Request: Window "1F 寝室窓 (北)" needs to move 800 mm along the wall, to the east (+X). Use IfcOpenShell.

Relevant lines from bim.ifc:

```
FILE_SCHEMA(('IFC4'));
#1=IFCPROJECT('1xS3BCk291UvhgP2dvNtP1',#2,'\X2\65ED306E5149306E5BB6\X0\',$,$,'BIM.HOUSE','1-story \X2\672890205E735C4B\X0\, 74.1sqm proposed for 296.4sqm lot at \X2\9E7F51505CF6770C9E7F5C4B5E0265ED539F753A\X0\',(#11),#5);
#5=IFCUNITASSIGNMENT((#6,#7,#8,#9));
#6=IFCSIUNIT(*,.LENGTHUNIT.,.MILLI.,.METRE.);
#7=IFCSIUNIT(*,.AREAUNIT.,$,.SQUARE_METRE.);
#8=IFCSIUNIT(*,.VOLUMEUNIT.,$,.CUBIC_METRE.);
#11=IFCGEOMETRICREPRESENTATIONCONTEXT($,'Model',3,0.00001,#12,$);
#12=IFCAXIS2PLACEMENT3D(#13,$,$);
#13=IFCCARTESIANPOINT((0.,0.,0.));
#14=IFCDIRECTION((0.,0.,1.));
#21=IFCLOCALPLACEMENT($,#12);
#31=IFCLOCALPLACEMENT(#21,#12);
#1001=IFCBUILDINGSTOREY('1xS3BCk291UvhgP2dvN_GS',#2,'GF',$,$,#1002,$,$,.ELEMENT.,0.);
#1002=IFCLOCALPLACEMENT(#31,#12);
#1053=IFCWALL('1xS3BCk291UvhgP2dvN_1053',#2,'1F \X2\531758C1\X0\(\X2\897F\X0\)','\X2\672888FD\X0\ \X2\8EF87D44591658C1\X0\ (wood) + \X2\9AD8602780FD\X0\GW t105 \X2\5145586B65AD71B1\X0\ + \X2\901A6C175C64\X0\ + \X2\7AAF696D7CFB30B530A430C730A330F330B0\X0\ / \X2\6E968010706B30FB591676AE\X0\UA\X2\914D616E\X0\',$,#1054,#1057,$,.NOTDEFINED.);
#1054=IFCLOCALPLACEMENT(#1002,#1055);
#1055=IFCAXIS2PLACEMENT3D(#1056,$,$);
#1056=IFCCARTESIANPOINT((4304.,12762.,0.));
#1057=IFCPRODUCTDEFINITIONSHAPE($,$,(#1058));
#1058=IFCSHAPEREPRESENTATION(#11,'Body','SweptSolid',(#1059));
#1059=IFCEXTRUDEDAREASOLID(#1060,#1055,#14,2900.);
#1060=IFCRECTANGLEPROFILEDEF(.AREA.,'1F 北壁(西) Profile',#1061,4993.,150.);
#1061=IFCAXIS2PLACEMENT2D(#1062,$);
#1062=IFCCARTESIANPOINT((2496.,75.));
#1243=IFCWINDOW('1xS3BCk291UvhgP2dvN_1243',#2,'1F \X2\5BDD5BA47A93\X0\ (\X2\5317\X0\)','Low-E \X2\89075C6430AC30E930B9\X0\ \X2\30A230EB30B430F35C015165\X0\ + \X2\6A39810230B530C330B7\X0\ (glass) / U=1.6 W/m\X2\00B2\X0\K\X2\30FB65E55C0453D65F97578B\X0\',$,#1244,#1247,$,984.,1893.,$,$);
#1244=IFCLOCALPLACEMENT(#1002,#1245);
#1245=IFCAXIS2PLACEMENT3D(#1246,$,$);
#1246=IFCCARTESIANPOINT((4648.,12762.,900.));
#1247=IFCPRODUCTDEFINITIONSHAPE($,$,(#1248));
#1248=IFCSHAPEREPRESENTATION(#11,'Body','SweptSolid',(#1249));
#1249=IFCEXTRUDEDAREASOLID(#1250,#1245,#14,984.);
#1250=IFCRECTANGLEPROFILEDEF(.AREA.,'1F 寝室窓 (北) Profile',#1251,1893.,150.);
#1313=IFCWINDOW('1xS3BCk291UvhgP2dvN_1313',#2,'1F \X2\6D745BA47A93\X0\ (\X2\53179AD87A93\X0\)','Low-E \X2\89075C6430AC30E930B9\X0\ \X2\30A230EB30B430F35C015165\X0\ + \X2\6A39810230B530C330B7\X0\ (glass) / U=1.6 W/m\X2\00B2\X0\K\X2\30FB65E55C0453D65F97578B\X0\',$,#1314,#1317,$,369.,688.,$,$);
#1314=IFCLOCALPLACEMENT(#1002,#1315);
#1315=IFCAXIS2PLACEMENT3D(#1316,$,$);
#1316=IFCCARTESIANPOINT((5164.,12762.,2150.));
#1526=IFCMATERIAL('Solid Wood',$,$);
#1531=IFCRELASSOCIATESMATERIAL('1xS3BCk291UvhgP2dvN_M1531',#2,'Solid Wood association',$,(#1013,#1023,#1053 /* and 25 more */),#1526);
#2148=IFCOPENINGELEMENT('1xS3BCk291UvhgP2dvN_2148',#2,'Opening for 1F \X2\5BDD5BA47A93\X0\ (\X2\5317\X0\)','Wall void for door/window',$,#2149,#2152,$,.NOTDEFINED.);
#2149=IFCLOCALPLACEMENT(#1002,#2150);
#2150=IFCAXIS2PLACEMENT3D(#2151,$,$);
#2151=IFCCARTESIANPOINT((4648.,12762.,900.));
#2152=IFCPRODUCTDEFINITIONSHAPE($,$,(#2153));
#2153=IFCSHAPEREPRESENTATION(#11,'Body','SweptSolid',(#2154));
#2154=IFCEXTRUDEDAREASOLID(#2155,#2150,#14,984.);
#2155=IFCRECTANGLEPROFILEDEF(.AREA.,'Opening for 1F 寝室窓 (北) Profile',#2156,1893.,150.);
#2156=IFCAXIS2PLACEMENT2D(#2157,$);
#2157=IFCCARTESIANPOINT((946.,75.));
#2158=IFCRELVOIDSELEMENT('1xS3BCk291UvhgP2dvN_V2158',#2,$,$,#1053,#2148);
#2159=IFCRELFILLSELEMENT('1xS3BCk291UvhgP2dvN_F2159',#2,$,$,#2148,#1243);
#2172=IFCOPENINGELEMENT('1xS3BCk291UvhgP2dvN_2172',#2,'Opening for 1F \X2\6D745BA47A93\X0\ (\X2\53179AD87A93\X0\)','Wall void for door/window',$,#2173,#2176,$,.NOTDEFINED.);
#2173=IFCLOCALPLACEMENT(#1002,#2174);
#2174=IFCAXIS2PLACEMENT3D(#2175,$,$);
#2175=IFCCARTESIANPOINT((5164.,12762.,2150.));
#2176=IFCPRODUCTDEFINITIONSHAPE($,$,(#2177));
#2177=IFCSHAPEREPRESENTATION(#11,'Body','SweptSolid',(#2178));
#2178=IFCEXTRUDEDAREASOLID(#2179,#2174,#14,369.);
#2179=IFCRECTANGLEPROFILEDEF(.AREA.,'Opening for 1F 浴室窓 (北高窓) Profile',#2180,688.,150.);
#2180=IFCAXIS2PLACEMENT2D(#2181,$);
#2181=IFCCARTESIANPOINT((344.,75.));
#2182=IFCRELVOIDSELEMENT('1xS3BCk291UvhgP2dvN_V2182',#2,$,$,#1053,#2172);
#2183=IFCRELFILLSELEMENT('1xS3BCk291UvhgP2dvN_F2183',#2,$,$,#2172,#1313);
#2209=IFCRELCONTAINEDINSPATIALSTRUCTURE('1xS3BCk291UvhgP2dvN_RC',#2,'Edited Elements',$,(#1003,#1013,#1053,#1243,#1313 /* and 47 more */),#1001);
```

```python
import ifcopenshell
import ifcopenshell.api.geometry
import ifcopenshell.util.placement
import ifcopenshell.util.unit

model = ifcopenshell.open("bim.ifc")
unit_scale = ifcopenshell.util.unit.calculate_unit_scale(model)

window = model.by_guid("1xS3BCk291UvhgP2dvN_1243")
opening = window.FillsVoids[0].RelatingOpeningElement
wall = opening.VoidsElements[0].RelatingBuildingElement

wall_matrix = ifcopenshell.util.placement.get_local_placement(wall.ObjectPlacement)
shift = wall_matrix[:3, 0] * 0.8 / unit_scale
before = ifcopenshell.util.placement.get_local_placement(window.ObjectPlacement)[:3, 3].copy()

# The window is not placed relative to its opening, so move both.
for product in (opening, window):
    matrix = ifcopenshell.util.placement.get_local_placement(product.ObjectPlacement)
    matrix[:3, 3] += shift
    ifcopenshell.api.geometry.edit_object_placement(model, product=product, matrix=matrix, is_si=False)

after = ifcopenshell.util.placement.get_local_placement(window.ObjectPlacement)[:3, 3]
print("window moved by", (after - before).round(3) + 0.0)

model.write("bim_v2.ifc")
```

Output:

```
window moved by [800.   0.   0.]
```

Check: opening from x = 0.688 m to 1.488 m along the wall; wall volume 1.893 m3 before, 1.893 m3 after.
